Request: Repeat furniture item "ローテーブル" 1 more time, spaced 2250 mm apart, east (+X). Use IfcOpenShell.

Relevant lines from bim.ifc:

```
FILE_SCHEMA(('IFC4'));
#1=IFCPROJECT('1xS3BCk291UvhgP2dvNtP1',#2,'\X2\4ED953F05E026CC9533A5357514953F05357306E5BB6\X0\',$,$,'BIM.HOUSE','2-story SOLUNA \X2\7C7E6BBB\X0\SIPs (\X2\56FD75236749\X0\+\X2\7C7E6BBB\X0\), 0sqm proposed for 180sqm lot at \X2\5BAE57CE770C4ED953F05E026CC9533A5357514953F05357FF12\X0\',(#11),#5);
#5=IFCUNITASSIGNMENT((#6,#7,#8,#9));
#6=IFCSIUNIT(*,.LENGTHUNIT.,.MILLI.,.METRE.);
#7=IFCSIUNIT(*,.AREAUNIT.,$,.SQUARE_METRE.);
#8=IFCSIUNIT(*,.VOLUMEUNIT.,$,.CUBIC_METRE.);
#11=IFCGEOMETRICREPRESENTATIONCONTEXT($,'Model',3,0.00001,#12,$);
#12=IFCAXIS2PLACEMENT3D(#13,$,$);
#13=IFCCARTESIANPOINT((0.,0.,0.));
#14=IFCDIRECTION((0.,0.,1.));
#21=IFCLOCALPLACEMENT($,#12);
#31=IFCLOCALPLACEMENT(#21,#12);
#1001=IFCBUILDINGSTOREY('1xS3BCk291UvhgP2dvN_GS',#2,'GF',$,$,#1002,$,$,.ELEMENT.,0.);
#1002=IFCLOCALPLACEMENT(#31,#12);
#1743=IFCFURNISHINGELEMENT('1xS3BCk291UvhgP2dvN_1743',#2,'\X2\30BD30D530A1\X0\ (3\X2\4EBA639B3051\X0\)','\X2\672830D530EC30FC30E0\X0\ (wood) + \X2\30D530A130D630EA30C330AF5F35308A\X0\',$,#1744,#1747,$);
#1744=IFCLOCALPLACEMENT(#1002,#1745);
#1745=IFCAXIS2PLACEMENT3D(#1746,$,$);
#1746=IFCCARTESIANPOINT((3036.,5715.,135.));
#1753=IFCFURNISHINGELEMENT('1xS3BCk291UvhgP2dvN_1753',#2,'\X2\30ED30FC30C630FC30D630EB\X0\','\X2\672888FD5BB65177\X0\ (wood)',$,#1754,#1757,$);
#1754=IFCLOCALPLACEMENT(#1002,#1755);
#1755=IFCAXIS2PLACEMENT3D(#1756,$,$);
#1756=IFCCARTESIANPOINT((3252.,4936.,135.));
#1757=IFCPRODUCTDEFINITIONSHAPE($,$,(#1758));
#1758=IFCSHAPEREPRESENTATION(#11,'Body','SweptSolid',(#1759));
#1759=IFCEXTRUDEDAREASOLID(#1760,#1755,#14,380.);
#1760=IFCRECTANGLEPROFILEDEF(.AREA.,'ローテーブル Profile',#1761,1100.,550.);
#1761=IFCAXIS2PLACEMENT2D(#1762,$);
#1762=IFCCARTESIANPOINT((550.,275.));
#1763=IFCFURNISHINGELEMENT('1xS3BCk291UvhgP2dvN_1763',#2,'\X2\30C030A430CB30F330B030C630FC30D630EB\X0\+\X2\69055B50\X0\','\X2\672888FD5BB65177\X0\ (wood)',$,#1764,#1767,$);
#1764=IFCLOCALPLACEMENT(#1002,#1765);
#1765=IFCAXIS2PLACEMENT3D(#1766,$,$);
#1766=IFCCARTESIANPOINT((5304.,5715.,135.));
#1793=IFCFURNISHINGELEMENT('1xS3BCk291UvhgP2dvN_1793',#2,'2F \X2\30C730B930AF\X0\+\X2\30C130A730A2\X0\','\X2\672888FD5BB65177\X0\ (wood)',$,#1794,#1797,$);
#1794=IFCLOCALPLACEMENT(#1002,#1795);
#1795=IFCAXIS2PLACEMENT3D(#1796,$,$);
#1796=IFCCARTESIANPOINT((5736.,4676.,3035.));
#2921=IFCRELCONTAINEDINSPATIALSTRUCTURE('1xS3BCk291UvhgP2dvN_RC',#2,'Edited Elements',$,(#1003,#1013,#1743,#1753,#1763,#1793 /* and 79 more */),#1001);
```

```python
import numpy as np
import ifcopenshell
import ifcopenshell.api.geometry
import ifcopenshell.api.root
import ifcopenshell.util.element
import ifcopenshell.util.placement
import ifcopenshell.util.unit

model = ifcopenshell.open("bim.ifc")
unit_scale = ifcopenshell.util.unit.calculate_unit_scale(model)


def reuse_history(source, copy):
    """copy_class also copies each property set's owner history, people and application; keep the originals."""
    for rel in copy.IsDefinedBy:
        if rel.is_a("IfcRelDefinesByProperties") and (history := rel.RelatingPropertyDefinition.OwnerHistory):
            rel.RelatingPropertyDefinition.OwnerHistory = source.OwnerHistory
            ifcopenshell.util.element.remove_deep2(model, history)


source = model.by_guid("1xS3BCk291UvhgP2dvN_1753")
base = ifcopenshell.util.placement.get_local_placement(source.ObjectPlacement)
step = np.array([1.0, 0.0, 0.0]) * 2.25 / unit_scale

for i in range(1, 2):
    copy = ifcopenshell.api.root.copy_class(model, product=source)
    copy.Representation = ifcopenshell.util.element.copy_deep(
        model, source.Representation, exclude=["IfcGeometricRepresentationContext", "IfcRepresentationMap"]
    )
    reuse_history(source, copy)
    matrix = base.copy()
    matrix[:3, 3] += i * step
    print("added at", matrix[:3, 3].round(3) + 0.0)
    ifcopenshell.api.geometry.edit_object_placement(model, product=copy, matrix=matrix, is_si=False)

model.write("bim_updated.ifc")
```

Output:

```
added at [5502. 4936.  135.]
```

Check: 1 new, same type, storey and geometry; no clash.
